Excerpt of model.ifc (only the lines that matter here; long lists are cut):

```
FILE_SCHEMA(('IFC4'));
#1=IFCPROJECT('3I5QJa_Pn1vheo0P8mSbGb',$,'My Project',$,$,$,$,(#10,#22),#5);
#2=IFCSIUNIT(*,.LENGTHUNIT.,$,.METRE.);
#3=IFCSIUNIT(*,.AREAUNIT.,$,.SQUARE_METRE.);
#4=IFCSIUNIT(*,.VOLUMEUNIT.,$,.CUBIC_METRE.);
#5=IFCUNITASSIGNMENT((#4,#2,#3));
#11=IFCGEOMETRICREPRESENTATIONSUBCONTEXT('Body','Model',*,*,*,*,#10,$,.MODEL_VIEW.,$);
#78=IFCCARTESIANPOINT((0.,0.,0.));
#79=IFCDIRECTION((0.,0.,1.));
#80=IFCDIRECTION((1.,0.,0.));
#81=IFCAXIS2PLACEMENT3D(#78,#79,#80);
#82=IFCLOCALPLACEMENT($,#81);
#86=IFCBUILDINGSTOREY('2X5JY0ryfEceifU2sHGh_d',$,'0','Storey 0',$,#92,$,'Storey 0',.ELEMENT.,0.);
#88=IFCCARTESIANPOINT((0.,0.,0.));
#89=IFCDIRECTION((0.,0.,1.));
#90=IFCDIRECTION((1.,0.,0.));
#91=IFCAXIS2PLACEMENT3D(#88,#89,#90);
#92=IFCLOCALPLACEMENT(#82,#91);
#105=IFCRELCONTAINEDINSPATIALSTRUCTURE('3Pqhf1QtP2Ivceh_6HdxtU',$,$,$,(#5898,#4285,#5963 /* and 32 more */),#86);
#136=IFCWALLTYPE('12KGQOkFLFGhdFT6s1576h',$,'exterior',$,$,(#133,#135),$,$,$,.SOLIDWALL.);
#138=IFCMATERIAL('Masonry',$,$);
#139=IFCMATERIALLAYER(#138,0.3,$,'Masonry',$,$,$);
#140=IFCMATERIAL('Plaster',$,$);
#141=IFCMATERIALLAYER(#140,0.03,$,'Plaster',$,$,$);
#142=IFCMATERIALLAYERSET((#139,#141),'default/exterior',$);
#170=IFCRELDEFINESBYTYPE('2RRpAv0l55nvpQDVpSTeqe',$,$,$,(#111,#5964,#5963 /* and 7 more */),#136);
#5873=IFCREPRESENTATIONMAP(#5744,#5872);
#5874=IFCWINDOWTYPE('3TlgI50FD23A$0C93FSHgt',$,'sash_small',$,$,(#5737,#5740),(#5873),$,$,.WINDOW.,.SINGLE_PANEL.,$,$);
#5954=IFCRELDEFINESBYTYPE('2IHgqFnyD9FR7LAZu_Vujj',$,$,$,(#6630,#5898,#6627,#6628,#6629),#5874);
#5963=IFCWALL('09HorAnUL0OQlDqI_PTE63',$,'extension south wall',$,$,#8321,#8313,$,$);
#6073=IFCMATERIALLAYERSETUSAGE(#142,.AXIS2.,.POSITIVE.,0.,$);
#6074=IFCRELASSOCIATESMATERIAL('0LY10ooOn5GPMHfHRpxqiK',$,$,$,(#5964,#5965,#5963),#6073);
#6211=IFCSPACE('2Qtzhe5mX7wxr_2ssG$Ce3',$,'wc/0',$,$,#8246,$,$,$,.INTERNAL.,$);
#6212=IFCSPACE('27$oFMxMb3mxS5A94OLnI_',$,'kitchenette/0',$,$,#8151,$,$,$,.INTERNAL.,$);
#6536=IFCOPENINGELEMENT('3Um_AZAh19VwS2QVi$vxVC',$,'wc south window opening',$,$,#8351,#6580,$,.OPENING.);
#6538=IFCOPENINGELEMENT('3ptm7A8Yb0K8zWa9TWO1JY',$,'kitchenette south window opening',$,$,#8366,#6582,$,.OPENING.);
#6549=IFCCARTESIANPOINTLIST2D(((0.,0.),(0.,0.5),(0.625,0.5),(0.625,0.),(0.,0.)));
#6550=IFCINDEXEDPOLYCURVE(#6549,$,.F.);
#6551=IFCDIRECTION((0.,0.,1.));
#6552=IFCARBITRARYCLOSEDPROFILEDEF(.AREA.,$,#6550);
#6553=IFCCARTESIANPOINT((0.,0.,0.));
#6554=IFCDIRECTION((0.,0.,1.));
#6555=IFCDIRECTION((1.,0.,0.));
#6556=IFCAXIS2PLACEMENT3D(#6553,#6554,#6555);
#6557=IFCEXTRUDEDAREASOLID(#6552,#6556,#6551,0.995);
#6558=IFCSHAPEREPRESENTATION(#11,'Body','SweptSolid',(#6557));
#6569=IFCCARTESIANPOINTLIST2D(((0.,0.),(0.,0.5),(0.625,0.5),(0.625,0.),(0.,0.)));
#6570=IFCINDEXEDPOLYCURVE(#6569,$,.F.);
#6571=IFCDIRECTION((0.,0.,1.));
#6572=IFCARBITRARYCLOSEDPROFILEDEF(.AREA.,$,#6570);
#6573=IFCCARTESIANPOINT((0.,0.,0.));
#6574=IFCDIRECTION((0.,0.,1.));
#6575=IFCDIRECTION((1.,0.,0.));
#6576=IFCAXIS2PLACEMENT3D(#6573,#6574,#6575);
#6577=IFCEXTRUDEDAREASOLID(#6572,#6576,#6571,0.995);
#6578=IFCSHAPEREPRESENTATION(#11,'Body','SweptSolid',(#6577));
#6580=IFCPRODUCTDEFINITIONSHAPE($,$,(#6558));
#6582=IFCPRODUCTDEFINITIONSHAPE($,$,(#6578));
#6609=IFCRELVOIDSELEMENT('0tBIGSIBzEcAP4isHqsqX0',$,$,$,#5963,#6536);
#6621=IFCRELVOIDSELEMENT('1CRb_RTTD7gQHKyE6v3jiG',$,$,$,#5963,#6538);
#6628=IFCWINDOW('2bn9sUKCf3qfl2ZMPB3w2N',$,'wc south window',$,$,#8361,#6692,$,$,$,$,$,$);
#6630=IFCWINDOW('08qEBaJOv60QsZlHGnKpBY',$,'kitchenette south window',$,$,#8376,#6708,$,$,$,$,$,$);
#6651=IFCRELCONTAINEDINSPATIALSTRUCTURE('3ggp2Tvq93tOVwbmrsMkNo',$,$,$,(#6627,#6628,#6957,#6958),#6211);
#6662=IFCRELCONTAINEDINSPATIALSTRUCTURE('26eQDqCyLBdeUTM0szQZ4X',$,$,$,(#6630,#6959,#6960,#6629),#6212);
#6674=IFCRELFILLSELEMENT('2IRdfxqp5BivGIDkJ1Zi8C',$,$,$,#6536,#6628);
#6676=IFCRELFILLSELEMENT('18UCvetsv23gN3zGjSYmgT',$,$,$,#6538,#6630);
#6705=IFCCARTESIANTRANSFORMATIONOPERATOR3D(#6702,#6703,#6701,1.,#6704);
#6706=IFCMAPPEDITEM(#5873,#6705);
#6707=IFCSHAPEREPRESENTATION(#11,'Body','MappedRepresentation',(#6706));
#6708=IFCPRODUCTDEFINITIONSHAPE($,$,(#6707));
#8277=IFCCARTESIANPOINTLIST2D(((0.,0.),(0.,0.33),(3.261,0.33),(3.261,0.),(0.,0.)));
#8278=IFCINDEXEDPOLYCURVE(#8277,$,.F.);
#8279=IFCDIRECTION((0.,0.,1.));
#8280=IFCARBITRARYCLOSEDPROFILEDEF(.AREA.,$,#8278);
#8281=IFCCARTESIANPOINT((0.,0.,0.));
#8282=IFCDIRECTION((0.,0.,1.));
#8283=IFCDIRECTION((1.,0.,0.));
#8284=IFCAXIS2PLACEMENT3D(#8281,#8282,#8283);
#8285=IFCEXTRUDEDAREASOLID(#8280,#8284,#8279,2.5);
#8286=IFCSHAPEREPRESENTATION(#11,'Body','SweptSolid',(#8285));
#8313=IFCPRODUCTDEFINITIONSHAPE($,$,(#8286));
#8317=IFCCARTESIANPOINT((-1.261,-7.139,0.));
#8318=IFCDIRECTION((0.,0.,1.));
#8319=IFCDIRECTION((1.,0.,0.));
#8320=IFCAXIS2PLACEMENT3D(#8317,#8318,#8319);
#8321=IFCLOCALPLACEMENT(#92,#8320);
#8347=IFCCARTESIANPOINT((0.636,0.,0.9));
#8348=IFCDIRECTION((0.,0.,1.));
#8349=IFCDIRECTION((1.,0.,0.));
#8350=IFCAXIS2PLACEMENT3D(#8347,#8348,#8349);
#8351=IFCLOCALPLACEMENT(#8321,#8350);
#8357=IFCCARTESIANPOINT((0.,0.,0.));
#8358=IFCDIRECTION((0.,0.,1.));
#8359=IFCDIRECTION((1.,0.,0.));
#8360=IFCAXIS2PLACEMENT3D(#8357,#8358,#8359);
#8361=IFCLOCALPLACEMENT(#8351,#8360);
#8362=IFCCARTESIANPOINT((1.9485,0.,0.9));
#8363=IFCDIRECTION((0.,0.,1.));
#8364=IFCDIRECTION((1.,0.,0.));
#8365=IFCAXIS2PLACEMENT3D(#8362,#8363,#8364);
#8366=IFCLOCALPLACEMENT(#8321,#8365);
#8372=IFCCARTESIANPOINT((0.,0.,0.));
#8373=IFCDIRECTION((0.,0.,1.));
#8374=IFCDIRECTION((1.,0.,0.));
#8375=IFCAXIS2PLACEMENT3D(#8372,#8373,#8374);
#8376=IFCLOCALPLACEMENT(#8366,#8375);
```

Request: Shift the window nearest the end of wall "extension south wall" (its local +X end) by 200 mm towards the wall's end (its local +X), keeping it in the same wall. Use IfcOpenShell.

```python
import ifcopenshell
import ifcopenshell.api.geometry
import ifcopenshell.util.placement
import ifcopenshell.util.unit

model = ifcopenshell.open("model.ifc")
unit_scale = ifcopenshell.util.unit.calculate_unit_scale(model)

window = model.by_guid("08qEBaJOv60QsZlHGnKpBY")
opening = window.FillsVoids[0].RelatingOpeningElement
wall = opening.VoidsElements[0].RelatingBuildingElement

wall_matrix = ifcopenshell.util.placement.get_local_placement(wall.ObjectPlacement)
shift = wall_matrix[:3, 0] * 0.2 / unit_scale
before = ifcopenshell.util.placement.get_local_placement(window.ObjectPlacement)[:3, 3].copy()

# The window is placed relative to its opening, so it follows when the opening moves.
matrix = ifcopenshell.util.placement.get_local_placement(opening.ObjectPlacement)
matrix[:3, 3] += shift
ifcopenshell.api.geometry.edit_object_placement(
    model, product=opening, matrix=matrix, is_si=False, should_transform_children=True
)

after = ifcopenshell.util.placement.get_local_placement(window.ObjectPlacement)[:3, 3]
print("window moved by", (after - before).round(3) + 0.0)

model.write("model_updated.ifc")
```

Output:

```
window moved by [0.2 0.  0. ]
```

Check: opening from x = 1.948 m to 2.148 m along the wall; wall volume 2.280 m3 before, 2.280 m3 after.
